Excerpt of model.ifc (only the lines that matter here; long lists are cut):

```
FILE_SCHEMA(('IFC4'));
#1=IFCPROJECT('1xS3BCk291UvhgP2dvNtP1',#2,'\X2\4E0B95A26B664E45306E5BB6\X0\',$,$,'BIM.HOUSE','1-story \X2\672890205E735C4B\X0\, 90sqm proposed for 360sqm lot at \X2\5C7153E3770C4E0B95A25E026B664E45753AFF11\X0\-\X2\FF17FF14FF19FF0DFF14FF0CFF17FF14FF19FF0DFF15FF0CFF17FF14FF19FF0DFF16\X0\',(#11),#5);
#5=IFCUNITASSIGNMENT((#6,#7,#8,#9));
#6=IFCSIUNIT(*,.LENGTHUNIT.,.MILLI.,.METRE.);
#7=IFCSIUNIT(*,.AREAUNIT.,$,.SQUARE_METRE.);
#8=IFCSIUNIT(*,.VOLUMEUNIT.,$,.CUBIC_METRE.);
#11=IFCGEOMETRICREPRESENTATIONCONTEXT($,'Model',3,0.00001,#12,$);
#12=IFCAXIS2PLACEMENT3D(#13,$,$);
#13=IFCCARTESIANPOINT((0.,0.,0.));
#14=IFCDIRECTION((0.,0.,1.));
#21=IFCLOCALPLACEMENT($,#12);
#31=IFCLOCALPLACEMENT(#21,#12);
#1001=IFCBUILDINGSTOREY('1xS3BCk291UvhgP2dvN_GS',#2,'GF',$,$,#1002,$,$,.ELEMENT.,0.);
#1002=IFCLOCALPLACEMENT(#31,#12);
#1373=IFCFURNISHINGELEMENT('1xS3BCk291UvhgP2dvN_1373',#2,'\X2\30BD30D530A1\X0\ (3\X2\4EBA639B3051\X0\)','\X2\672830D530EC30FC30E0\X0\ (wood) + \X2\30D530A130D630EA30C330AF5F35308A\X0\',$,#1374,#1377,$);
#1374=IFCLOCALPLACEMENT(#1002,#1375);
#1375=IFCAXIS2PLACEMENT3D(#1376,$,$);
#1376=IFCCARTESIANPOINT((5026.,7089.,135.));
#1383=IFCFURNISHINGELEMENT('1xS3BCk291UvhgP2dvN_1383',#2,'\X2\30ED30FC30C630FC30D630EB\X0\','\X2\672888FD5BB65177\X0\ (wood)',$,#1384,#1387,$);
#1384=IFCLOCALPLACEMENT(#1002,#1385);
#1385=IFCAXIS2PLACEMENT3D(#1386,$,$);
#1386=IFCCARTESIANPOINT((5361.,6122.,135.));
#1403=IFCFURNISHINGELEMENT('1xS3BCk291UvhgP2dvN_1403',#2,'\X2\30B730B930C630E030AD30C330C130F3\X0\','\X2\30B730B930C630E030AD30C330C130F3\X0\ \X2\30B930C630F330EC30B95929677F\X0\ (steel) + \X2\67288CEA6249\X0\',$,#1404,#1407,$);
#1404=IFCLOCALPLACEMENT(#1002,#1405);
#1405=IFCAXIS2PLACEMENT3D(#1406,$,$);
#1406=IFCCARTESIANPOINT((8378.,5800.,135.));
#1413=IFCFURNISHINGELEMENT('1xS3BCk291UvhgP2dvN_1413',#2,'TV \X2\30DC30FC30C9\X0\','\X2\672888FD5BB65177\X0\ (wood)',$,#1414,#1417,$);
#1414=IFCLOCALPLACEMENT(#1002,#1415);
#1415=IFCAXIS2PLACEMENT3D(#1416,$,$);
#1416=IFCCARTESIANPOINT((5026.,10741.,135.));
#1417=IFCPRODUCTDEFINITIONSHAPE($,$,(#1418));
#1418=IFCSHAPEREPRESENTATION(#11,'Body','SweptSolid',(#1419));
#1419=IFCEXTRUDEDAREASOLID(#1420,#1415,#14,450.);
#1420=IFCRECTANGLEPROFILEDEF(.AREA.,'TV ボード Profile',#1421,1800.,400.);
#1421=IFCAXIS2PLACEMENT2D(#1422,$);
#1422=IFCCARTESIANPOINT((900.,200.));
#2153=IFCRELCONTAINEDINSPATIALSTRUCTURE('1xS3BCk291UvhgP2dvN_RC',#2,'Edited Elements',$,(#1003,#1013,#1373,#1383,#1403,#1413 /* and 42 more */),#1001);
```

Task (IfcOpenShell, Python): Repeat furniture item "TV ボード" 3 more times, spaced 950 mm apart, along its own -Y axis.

```python
import ifcopenshell
import ifcopenshell.api.geometry
import ifcopenshell.api.root
import ifcopenshell.util.element
import ifcopenshell.util.placement
import ifcopenshell.util.unit

model = ifcopenshell.open("model.ifc")
unit_scale = ifcopenshell.util.unit.calculate_unit_scale(model)


def reuse_history(source, copy):
    """copy_class also copies each property set's owner history, people and application; keep the originals."""
    for rel in copy.IsDefinedBy:
        if rel.is_a("IfcRelDefinesByProperties") and (history := rel.RelatingPropertyDefinition.OwnerHistory):
            rel.RelatingPropertyDefinition.OwnerHistory = source.OwnerHistory
            ifcopenshell.util.element.remove_deep2(model, history)


source = model.by_id(1413)
base = ifcopenshell.util.placement.get_local_placement(source.ObjectPlacement)
step = -base[:3, 1] * 0.95 / unit_scale

for i in range(1, 4):
    copy = ifcopenshell.api.root.copy_class(model, product=source)
    copy.Representation = ifcopenshell.util.element.copy_deep(
        model, source.Representation, exclude=["IfcGeometricRepresentationContext", "IfcRepresentationMap"]
    )
    reuse_history(source, copy)
    matrix = base.copy()
    matrix[:3, 3] += i * step
    print("added at", matrix[:3, 3].round(3) + 0.0)
    ifcopenshell.api.geometry.edit_object_placement(model, product=copy, matrix=matrix, is_si=False)

model.write("model_updated.ifc")
```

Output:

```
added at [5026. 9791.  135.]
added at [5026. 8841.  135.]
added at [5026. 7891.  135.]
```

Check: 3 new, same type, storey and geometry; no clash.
